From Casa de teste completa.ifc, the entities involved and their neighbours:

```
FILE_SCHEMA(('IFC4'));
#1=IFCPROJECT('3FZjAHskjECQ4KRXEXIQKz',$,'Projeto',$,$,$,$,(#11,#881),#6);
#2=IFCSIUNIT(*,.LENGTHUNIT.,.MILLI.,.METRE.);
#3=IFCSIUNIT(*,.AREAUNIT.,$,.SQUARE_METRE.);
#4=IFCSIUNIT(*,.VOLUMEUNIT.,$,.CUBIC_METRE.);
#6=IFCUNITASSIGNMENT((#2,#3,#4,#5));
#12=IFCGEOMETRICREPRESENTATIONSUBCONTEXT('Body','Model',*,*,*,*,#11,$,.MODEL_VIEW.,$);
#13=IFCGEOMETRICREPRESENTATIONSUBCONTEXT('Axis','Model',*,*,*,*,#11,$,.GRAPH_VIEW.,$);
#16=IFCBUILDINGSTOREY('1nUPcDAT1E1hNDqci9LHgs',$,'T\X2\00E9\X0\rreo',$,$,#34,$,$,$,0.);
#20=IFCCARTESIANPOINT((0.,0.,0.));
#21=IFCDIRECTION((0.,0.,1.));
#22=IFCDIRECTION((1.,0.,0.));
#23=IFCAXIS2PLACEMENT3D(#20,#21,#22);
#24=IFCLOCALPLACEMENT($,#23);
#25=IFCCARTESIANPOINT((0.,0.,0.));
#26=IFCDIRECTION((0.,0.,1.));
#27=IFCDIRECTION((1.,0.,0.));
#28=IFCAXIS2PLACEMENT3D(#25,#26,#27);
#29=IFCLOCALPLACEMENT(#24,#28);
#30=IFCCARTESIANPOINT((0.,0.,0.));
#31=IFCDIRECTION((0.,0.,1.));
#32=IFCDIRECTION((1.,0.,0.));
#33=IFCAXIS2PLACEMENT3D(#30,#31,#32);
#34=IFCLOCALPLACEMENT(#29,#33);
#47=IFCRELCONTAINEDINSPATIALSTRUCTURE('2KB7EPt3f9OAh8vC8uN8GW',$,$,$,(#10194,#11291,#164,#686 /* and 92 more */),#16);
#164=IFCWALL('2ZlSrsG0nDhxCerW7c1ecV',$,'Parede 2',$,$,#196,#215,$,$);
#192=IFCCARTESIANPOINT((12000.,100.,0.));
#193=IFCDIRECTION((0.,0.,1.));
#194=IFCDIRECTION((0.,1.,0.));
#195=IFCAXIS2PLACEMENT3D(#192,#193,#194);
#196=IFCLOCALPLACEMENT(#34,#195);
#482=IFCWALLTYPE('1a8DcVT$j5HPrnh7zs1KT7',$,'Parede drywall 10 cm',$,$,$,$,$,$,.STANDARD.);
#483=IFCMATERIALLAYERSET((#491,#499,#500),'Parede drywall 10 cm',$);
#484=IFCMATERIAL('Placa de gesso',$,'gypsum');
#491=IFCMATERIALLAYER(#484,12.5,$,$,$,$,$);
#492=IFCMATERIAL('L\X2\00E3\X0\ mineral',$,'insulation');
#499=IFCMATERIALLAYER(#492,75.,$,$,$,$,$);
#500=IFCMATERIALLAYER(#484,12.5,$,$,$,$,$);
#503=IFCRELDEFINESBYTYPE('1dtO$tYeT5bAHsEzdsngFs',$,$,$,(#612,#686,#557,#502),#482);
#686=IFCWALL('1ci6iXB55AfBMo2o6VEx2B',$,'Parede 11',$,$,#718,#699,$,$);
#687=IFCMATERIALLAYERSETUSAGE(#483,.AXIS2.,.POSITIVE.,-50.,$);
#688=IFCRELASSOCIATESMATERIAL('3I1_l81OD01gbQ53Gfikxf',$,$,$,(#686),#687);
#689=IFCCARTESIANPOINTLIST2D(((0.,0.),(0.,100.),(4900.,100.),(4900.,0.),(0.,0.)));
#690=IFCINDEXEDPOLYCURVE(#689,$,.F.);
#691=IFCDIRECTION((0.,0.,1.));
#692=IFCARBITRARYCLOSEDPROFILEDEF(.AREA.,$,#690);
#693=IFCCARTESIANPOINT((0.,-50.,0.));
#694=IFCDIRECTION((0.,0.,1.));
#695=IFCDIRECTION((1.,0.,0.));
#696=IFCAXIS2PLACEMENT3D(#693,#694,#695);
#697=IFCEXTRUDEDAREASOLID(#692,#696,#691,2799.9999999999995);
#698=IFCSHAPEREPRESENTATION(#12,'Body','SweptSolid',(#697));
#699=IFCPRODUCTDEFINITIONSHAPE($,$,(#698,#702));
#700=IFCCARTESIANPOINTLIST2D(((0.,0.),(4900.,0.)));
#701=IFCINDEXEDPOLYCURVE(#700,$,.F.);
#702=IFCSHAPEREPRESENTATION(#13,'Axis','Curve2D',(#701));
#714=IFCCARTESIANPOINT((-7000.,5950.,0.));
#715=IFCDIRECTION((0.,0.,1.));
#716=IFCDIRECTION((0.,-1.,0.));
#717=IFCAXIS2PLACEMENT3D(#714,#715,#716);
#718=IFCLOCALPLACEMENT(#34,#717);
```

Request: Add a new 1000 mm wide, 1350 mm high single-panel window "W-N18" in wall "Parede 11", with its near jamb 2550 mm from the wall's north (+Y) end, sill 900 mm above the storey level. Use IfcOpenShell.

```python
import numpy as np
import ifcopenshell
import ifcopenshell.api.feature
import ifcopenshell.api.geometry
import ifcopenshell.api.root
import ifcopenshell.api.spatial
import ifcopenshell.geom
import ifcopenshell.util.element
import ifcopenshell.util.placement
import ifcopenshell.util.representation
import ifcopenshell.util.shape
import ifcopenshell.util.unit

model = ifcopenshell.open("Casa de teste completa.ifc")
unit_scale = ifcopenshell.util.unit.calculate_unit_scale(model)
settings = ifcopenshell.geom.settings()


def volume(element):
    """Net volume in cubic metres, openings subtracted."""
    shape = ifcopenshell.geom.create_shape(settings, element)
    return ifcopenshell.util.shape.get_volume(shape.geometry)


wall = model.by_guid("1ci6iXB55AfBMo2o6VEx2B")
storey = ifcopenshell.util.element.get_container(wall, ifc_class="IfcBuildingStorey")
context = ifcopenshell.util.representation.get_context(model, "Model", "Body", "MODEL_VIEW")
before = volume(wall)

width, height, from_end, sill = 1, 1.35, 2.55, 0.9  # metres

# The wall runs along its own X axis, and the end named is its -X end.
wall_shape = ifcopenshell.geom.create_shape(settings, wall)
x, y, z = ifcopenshell.util.shape.get_vertices(wall_shape.geometry).T
start = x.min() + from_end
face, thickness = float(y.min()), float(y.max() - y.min())
wall_matrix = ifcopenshell.util.placement.get_local_placement(wall.ObjectPlacement)
level = ifcopenshell.util.placement.get_local_placement(storey.ObjectPlacement)[2, 3]


def in_wall(x, y):
    """Placement at x, y metres in the wall's axes, at sill height."""
    matrix = wall_matrix.copy()
    matrix[:, 3] = wall_matrix @ np.array([x / unit_scale, y / unit_scale, 0.0, 1.0])
    matrix[2, 3] = level + sill / unit_scale
    return matrix


# Opening: a box that overshoots both wall faces by 50 mm.
opening = ifcopenshell.api.root.create_entity(model, ifc_class="IfcOpeningElement", predefined_type="OPENING")
box = ifcopenshell.api.geometry.add_wall_representation(
    model, context=context, length=width, height=height, thickness=thickness + 0.1
)
ifcopenshell.api.geometry.assign_representation(model, product=opening, representation=box)
ifcopenshell.api.geometry.edit_object_placement(model, product=opening, matrix=in_wall(start, face - 0.05), is_si=False)
ifcopenshell.api.feature.add_feature(model, feature=opening, element=wall)

window = ifcopenshell.api.root.create_entity(model, ifc_class="IfcWindow", name="W-N18", predefined_type="WINDOW")
window.OverallWidth, window.OverallHeight = width / unit_scale, height / unit_scale
window.PartitioningType = "SINGLE_PANEL"
body = ifcopenshell.api.geometry.add_window_representation(
    model,
    context=context,
    overall_width=window.OverallWidth,
    overall_height=window.OverallHeight,
    partition_type="SINGLE_PANEL",
)
ifcopenshell.api.geometry.assign_representation(model, product=window, representation=body)
ifcopenshell.api.spatial.assign_container(model, products=[window], relating_structure=storey)
ifcopenshell.api.feature.add_filling(model, opening=opening, element=window)

# Centre the window in the wall's thickness.
ifcopenshell.api.geometry.edit_object_placement(model, product=window, matrix=in_wall(start, face), is_si=False)
window_shape = ifcopenshell.geom.create_shape(settings, window)
depth = ifcopenshell.util.shape.get_vertices(window_shape.geometry)[:, 1]
offset = face + thickness / 2 - (depth.min() + depth.max()) / 2
ifcopenshell.api.geometry.edit_object_placement(model, product=window, matrix=in_wall(start, offset), is_si=False)

after = volume(wall)

print(f"wall volume {before:.3f} -> {after:.3f} m3")

model.write("Casa de teste completa_rev.ifc")
```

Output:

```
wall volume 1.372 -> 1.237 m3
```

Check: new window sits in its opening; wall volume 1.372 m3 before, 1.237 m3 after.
